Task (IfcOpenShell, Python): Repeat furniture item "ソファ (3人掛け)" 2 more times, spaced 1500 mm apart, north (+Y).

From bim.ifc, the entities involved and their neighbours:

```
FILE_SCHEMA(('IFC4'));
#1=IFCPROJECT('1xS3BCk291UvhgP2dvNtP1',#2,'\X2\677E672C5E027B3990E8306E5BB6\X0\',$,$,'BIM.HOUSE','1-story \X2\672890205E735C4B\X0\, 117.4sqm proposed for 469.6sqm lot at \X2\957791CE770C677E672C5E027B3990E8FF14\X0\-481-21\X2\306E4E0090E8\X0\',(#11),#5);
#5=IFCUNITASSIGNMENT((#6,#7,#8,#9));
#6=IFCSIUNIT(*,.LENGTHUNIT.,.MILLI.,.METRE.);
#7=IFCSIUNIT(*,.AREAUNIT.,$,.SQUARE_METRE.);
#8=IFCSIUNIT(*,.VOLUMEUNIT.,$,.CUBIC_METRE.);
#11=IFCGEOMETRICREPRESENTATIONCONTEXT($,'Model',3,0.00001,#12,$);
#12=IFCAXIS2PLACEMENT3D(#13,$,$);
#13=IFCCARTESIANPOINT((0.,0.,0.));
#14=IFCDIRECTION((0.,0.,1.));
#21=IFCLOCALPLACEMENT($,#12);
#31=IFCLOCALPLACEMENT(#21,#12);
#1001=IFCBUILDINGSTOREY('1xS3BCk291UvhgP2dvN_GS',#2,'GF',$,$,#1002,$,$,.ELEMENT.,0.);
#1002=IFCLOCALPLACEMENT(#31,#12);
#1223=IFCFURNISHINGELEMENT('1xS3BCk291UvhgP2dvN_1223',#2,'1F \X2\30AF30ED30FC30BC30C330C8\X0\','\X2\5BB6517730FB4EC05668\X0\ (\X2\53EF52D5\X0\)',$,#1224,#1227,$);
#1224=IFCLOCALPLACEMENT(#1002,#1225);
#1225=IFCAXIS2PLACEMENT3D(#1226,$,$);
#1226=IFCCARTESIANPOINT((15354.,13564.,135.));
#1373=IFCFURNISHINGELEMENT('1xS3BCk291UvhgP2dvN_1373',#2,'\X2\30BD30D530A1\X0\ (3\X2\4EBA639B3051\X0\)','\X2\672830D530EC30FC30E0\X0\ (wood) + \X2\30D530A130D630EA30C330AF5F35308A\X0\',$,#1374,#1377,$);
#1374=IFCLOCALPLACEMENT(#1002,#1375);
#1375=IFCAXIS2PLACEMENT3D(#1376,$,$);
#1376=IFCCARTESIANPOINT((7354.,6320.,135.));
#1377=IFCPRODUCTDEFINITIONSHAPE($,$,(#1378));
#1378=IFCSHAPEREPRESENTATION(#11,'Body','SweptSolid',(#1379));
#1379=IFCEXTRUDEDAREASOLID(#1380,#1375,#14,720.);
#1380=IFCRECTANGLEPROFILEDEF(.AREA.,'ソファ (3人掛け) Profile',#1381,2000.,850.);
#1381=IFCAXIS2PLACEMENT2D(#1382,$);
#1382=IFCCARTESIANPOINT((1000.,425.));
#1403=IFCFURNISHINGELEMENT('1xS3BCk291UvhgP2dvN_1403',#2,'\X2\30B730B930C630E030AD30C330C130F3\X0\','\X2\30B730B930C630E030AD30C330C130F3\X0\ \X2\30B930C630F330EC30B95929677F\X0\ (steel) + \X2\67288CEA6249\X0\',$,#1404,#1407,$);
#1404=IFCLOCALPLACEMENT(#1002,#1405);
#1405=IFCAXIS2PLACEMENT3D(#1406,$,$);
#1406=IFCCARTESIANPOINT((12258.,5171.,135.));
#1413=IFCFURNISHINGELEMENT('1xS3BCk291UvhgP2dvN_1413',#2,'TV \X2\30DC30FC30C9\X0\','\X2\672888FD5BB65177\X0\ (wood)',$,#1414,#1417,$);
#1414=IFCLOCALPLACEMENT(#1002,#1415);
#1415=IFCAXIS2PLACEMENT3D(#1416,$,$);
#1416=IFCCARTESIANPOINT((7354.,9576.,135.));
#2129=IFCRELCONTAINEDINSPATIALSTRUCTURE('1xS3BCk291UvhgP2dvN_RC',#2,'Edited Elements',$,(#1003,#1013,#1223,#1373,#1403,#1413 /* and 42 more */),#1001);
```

```python
import numpy as np
import ifcopenshell
import ifcopenshell.api.geometry
import ifcopenshell.api.root
import ifcopenshell.util.element
import ifcopenshell.util.placement

model = ifcopenshell.open("bim.ifc")


def reuse_history(source, copy):
    """copy_class also copies each property set's owner history, people and application; keep the originals."""
    for rel in copy.IsDefinedBy:
        if rel.is_a("IfcRelDefinesByProperties") and (history := rel.RelatingPropertyDefinition.OwnerHistory):
            rel.RelatingPropertyDefinition.OwnerHistory = source.OwnerHistory
            ifcopenshell.util.element.remove_deep2(model, history)


source = model.by_id(1373)
base = ifcopenshell.util.placement.get_local_placement(source.ObjectPlacement)
step = np.array([0.0, 1.0, 0.0]) * 1500.0

for i in range(1, 3):
    copy = ifcopenshell.api.root.copy_class(model, product=source)
    copy.Representation = ifcopenshell.util.element.copy_deep(
        model, source.Representation, exclude=["IfcGeometricRepresentationContext", "IfcRepresentationMap"]
    )
    reuse_history(source, copy)
    matrix = base.copy()
    matrix[:3, 3] += i * step
    print("added at", matrix[:3, 3].round(3) + 0.0)
    ifcopenshell.api.geometry.edit_object_placement(model, product=copy, matrix=matrix, is_si=False)

model.write("bim_rev.ifc")
```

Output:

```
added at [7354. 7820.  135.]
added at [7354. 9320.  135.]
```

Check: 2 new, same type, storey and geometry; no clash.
